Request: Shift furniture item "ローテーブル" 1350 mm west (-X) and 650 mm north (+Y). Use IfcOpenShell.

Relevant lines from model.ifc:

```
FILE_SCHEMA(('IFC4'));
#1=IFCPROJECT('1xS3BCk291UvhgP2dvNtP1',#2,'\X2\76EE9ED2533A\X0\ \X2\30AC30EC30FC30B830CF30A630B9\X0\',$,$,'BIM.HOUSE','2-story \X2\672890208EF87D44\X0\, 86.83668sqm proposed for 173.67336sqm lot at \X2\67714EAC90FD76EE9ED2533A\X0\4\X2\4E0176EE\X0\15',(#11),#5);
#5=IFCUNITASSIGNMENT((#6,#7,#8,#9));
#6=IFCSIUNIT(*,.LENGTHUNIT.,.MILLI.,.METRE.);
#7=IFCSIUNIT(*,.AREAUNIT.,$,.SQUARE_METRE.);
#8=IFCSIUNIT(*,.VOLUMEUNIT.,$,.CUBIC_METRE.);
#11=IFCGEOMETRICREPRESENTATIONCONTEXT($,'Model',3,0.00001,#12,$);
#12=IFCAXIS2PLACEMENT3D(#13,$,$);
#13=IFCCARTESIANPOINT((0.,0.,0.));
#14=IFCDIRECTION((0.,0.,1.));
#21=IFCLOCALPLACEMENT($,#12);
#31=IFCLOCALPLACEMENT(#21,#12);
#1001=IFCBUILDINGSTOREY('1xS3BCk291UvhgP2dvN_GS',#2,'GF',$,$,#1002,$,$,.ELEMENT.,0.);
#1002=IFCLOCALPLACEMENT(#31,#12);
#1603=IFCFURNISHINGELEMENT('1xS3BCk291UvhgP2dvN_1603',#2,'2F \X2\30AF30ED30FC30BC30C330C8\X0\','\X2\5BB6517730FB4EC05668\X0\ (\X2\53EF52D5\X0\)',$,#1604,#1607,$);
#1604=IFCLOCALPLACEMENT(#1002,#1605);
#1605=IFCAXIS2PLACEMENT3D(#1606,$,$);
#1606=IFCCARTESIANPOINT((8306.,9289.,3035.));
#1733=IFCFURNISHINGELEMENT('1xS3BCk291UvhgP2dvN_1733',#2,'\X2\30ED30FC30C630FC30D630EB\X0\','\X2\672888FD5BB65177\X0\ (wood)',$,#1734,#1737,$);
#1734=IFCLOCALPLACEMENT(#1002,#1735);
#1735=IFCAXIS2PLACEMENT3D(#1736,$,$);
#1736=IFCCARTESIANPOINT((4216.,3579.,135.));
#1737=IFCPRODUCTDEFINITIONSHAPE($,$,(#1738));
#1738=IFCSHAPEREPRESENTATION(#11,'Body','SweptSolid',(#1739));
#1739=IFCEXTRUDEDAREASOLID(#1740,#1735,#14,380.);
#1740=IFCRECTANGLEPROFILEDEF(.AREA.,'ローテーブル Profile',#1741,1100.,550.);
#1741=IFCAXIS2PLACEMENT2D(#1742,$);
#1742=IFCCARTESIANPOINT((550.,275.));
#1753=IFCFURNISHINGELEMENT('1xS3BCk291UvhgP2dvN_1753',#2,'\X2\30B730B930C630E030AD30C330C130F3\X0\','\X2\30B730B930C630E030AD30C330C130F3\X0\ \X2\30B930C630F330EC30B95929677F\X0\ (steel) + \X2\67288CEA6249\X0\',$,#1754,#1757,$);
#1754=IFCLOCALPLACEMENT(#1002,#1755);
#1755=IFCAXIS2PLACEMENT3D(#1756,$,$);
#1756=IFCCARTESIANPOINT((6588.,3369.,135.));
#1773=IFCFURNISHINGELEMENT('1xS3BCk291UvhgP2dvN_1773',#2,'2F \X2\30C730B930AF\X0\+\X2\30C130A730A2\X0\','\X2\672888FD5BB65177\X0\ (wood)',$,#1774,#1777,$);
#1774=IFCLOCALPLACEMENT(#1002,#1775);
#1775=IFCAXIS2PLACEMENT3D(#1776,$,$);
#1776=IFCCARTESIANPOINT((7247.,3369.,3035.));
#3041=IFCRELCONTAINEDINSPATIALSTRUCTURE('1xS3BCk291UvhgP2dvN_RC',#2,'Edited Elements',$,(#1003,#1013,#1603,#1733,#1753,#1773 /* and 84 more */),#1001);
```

```python
import ifcopenshell
import ifcopenshell.api.geometry
import ifcopenshell.util.placement
import ifcopenshell.util.unit

model = ifcopenshell.open("model.ifc")
unit_scale = ifcopenshell.util.unit.calculate_unit_scale(model)

item = model.by_guid("1xS3BCk291UvhgP2dvN_1733")
matrix = ifcopenshell.util.placement.get_local_placement(item.ObjectPlacement)
matrix[0, 3] -= 1.35 / unit_scale
matrix[1, 3] += 0.65 / unit_scale
ifcopenshell.api.geometry.edit_object_placement(model, product=item, matrix=matrix, is_si=False)

print(ifcopenshell.util.placement.get_local_placement(item.ObjectPlacement).round(3) + 0.0)

model.write("model_edited.ifc")
```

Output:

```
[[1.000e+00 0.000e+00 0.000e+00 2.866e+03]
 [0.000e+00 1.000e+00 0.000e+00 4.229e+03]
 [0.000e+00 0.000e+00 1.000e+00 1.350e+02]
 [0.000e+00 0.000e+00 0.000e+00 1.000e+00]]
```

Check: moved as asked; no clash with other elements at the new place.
